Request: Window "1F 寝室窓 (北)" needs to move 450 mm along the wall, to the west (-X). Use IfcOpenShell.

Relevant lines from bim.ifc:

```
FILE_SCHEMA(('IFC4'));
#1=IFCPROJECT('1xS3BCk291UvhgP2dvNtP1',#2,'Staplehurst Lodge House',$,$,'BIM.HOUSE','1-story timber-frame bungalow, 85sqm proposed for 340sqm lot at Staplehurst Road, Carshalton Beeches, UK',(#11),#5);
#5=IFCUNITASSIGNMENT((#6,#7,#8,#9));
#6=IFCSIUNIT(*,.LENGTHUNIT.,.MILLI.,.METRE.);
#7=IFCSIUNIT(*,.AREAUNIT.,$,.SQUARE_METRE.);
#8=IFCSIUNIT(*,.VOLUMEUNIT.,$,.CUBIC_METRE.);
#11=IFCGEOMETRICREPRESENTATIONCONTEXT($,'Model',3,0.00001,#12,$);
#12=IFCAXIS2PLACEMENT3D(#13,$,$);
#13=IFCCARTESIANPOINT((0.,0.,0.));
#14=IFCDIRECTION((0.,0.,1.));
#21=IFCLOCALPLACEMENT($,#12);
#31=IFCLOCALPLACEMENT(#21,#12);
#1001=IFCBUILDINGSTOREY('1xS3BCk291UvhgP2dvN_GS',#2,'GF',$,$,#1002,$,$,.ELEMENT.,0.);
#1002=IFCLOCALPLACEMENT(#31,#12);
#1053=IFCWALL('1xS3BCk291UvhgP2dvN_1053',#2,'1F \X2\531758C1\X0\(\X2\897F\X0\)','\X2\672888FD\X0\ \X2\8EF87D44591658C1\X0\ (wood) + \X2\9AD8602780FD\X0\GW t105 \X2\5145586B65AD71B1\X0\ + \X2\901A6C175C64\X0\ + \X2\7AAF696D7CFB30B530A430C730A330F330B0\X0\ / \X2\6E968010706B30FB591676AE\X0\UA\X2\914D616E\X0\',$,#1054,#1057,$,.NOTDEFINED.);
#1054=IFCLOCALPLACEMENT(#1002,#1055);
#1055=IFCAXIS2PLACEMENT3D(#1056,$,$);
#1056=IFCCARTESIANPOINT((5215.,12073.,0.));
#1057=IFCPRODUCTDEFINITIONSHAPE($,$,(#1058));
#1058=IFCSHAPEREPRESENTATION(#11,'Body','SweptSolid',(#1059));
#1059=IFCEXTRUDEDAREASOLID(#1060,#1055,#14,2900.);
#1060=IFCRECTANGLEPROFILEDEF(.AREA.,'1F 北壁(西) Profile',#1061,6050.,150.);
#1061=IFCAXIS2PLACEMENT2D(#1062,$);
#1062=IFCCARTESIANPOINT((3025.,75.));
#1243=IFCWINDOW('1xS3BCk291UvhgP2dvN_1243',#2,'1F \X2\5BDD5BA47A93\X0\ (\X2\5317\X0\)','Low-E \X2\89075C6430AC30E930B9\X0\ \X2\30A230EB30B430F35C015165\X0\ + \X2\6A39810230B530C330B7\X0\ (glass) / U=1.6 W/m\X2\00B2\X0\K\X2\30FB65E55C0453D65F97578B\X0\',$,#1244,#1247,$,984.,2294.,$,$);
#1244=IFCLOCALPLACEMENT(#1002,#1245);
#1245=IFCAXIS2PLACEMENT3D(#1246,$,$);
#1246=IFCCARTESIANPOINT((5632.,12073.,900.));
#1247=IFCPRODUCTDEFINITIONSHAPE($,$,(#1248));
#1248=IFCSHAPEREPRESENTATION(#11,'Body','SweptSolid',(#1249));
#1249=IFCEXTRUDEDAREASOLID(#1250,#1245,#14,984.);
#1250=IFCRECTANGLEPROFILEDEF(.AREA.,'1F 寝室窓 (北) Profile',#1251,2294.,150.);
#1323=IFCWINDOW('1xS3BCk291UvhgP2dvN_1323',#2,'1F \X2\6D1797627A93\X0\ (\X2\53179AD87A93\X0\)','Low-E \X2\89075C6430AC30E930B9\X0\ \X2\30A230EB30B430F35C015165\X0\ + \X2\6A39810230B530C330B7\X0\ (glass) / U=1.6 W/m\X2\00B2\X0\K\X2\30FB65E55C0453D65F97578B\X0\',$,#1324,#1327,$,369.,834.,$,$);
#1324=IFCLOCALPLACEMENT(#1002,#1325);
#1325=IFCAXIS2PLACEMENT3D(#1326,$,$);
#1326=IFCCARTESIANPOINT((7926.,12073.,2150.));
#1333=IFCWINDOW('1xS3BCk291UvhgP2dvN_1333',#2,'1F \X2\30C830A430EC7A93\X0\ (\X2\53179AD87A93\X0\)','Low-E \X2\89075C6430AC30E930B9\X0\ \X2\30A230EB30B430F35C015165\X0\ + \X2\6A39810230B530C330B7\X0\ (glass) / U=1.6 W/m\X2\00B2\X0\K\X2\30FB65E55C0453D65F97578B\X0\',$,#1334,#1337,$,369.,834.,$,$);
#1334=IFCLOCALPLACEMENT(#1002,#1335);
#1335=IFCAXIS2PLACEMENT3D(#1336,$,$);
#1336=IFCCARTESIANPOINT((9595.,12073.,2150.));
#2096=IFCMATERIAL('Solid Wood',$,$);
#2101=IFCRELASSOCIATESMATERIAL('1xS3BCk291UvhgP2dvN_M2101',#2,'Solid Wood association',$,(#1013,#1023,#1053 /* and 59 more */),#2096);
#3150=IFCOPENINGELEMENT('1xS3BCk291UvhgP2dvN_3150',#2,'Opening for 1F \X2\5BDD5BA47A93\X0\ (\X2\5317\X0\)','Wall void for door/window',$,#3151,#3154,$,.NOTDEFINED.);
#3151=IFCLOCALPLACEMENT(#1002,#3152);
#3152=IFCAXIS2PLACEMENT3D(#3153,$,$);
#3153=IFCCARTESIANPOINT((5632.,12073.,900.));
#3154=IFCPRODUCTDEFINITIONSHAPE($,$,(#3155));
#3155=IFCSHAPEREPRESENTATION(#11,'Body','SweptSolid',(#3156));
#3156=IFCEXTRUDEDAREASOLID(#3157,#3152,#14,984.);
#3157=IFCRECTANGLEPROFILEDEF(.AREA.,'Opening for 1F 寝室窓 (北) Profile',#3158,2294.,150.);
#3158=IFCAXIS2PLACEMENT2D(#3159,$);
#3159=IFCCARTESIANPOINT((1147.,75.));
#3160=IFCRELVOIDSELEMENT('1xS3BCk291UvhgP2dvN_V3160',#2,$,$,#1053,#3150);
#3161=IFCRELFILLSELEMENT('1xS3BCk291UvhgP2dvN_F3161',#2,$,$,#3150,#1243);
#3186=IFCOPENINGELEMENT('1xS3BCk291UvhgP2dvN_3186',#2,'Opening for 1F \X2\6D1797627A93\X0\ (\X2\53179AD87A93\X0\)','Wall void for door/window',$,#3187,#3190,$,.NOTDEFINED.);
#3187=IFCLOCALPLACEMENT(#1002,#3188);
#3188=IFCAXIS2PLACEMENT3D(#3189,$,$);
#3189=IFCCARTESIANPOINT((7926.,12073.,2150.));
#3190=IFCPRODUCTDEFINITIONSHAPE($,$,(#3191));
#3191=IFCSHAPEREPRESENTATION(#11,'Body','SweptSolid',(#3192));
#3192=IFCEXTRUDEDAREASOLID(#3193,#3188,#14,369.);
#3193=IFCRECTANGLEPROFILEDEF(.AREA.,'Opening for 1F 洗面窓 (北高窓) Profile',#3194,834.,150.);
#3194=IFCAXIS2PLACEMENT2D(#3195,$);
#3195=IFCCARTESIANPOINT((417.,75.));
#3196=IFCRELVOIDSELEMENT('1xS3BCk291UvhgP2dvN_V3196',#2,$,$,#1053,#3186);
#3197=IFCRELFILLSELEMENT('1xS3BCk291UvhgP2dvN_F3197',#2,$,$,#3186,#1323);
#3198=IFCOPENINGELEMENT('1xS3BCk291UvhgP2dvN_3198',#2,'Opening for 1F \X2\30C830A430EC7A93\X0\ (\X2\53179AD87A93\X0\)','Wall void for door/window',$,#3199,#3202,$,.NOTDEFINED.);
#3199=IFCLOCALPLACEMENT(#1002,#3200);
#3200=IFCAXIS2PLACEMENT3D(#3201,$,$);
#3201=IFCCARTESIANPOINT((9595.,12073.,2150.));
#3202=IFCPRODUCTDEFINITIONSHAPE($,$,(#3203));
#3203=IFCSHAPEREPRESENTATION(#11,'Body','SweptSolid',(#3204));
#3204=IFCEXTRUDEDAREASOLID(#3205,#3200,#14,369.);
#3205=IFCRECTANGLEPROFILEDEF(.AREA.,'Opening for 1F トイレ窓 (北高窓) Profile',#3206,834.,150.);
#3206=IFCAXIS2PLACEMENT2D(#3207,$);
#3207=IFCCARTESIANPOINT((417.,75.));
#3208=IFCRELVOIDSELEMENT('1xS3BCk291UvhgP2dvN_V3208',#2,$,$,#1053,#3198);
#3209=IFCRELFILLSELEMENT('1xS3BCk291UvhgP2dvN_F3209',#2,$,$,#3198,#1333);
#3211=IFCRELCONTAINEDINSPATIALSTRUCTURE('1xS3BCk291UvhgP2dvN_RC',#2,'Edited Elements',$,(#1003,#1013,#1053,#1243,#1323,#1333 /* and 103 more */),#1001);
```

```python
import ifcopenshell
import ifcopenshell.api.geometry
import ifcopenshell.util.placement

model = ifcopenshell.open("bim.ifc")

window = model.by_guid("1xS3BCk291UvhgP2dvN_1243")
opening = window.FillsVoids[0].RelatingOpeningElement
wall = opening.VoidsElements[0].RelatingBuildingElement

wall_matrix = ifcopenshell.util.placement.get_local_placement(wall.ObjectPlacement)
shift = wall_matrix[:3, 0] * -450.0
before = ifcopenshell.util.placement.get_local_placement(window.ObjectPlacement)[:3, 3].copy()

# The window is not placed relative to its opening, so move both.
for product in (opening, window):
    matrix = ifcopenshell.util.placement.get_local_placement(product.ObjectPlacement)
    matrix[:3, 3] += shift
    ifcopenshell.api.geometry.edit_object_placement(model, product=product, matrix=matrix, is_si=False)

after = ifcopenshell.util.placement.get_local_placement(window.ObjectPlacement)[:3, 3]
print("window moved by", (after - before).round(3) + 0.0)

model.write("bim_rev.ifc")
```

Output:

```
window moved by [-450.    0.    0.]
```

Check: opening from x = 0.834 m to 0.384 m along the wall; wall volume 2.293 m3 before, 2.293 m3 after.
